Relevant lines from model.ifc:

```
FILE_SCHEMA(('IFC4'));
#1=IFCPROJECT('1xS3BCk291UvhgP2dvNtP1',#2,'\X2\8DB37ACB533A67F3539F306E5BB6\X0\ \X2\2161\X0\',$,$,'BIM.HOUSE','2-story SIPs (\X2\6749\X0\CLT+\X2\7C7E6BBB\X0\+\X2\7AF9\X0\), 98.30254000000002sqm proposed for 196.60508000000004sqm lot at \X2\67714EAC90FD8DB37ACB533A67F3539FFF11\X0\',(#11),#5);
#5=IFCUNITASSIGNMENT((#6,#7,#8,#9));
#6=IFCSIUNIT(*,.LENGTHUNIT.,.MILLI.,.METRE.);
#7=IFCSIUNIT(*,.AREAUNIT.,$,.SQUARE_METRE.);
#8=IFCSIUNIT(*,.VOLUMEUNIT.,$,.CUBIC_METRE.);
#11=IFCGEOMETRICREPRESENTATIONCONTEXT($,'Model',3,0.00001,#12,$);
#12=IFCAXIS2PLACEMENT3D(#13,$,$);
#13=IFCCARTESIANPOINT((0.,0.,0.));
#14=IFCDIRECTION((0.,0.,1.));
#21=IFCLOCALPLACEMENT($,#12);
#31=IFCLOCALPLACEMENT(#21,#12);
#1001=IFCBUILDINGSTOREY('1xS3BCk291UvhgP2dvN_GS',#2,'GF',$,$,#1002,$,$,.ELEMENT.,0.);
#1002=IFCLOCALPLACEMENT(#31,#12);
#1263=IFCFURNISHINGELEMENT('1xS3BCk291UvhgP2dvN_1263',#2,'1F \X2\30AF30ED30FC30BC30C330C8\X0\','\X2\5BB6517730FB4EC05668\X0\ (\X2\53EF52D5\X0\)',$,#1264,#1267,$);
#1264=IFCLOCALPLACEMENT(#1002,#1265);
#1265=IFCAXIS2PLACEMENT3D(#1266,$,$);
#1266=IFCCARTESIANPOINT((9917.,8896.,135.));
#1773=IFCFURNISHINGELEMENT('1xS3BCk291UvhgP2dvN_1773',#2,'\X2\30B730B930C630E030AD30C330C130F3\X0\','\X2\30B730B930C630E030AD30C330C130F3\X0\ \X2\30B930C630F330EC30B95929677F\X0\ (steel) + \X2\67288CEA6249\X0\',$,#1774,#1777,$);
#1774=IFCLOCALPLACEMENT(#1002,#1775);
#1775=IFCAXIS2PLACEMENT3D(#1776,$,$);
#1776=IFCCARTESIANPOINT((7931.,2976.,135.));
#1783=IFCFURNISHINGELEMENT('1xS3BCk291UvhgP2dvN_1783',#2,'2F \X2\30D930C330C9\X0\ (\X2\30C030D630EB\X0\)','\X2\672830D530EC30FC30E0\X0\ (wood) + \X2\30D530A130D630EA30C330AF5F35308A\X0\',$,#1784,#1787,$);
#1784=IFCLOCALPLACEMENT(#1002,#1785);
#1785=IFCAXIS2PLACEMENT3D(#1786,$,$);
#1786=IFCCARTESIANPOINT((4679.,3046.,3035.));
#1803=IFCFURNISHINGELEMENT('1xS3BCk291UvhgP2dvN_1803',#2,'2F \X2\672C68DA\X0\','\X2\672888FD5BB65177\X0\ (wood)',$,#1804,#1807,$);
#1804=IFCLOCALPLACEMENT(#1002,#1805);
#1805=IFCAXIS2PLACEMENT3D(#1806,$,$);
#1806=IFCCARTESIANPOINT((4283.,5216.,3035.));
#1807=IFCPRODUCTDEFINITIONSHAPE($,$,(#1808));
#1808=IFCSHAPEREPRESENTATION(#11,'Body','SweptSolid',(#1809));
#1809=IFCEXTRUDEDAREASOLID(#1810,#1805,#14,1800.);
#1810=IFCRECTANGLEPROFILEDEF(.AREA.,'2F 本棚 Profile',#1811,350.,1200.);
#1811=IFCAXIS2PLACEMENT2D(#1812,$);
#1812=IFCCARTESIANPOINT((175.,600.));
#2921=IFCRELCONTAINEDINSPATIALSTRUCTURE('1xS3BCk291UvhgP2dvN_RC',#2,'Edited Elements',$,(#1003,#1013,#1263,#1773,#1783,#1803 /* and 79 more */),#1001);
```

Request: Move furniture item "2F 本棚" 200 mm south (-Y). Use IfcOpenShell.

```python
import ifcopenshell
import ifcopenshell.api.geometry
import ifcopenshell.util.placement

model = ifcopenshell.open("model.ifc")

item = model.by_id(1803)
matrix = ifcopenshell.util.placement.get_local_placement(item.ObjectPlacement)
matrix[1, 3] -= 200.0
ifcopenshell.api.geometry.edit_object_placement(model, product=item, matrix=matrix, is_si=False)

print(ifcopenshell.util.placement.get_local_placement(item.ObjectPlacement).round(3) + 0.0)

model.write("model_v2.ifc")
```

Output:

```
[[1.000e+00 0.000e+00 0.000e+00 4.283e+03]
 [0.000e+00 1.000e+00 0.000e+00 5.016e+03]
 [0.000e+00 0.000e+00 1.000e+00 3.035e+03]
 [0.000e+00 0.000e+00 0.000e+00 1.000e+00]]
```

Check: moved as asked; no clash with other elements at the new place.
